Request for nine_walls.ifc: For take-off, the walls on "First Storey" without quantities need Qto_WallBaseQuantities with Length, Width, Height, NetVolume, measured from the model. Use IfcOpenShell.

First a look at what the model holds.

```python
import ifcopenshell
import ifcopenshell.util.element
import ifcopenshell.util.unit

model = ifcopenshell.open("nine_walls.ifc")
print(model.schema)
for unit_type in ("LENGTHUNIT", "AREAUNIT", "VOLUMEUNIT"):
    print(unit_type, ifcopenshell.util.unit.calculate_unit_scale(model, unit_type))
storey = next(s for s in model.by_type("IfcBuildingStorey") if s.Name == "First Storey")
walls = [e for e in ifcopenshell.util.element.get_decomposition(storey) if e.is_a("IfcWall")]
for e in sorted(walls, key=lambda e: e.id()):
    print(e.id(), e.is_a(), e.Name, list(ifcopenshell.util.element.get_psets(e, qtos_only=True)), sep=" | ")
```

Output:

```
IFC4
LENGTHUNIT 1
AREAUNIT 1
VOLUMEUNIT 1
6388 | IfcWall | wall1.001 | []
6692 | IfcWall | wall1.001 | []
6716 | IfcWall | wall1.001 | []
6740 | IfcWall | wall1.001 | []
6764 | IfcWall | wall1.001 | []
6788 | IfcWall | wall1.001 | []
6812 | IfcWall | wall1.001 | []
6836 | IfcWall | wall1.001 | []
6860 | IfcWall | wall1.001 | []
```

```python
import ifcopenshell
import ifcopenshell.api.pset
import ifcopenshell.geom
import ifcopenshell.util.element
import ifcopenshell.util.shape
import ifcopenshell.util.unit

model = ifcopenshell.open("nine_walls.ifc")
unit_scale = ifcopenshell.util.unit.calculate_unit_scale(model)
volume_scale = ifcopenshell.util.unit.calculate_unit_scale(model, "VOLUMEUNIT")
settings = ifcopenshell.geom.settings()

storey = next(s for s in model.by_type("IfcBuildingStorey") if s.Name == "First Storey")
walls = [e for e in ifcopenshell.util.element.get_decomposition(storey) if e.is_a("IfcWall")]

for e in sorted(walls, key=lambda e: e.id()):
    if ifcopenshell.util.element.get_psets(e, qtos_only=True, should_inherit=False):
        continue
    # Geometry comes back in metres, in the element's own axes.
    shape = ifcopenshell.geom.create_shape(settings, e)
    values = {
        "Length": ifcopenshell.util.shape.get_x(shape.geometry) / unit_scale,
        "Width": ifcopenshell.util.shape.get_y(shape.geometry) / unit_scale,
        "Height": ifcopenshell.util.shape.get_z(shape.geometry) / unit_scale,
        "NetVolume": ifcopenshell.util.shape.get_volume(shape.geometry) / volume_scale,
    }
    qto = ifcopenshell.api.pset.add_qto(model, product=e, name="Qto_WallBaseQuantities")
    ifcopenshell.api.pset.edit_qto(model, qto=qto, properties=values)
    print(e.id(), {k: round(v, 3) for k, v in values.items()})

model.write("nine_walls_rev.ifc")
```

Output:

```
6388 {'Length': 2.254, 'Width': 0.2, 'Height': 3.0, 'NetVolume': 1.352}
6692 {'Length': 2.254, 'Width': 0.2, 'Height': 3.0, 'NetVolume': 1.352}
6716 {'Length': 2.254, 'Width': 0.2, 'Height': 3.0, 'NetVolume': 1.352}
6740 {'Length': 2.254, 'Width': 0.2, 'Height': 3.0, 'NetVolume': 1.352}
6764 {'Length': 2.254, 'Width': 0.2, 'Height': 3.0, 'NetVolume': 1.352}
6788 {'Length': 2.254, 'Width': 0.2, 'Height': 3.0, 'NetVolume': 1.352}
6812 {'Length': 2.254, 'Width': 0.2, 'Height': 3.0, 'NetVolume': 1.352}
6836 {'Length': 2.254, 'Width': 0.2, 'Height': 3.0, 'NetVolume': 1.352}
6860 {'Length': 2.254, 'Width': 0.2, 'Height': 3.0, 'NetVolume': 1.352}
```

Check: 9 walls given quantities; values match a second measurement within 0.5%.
